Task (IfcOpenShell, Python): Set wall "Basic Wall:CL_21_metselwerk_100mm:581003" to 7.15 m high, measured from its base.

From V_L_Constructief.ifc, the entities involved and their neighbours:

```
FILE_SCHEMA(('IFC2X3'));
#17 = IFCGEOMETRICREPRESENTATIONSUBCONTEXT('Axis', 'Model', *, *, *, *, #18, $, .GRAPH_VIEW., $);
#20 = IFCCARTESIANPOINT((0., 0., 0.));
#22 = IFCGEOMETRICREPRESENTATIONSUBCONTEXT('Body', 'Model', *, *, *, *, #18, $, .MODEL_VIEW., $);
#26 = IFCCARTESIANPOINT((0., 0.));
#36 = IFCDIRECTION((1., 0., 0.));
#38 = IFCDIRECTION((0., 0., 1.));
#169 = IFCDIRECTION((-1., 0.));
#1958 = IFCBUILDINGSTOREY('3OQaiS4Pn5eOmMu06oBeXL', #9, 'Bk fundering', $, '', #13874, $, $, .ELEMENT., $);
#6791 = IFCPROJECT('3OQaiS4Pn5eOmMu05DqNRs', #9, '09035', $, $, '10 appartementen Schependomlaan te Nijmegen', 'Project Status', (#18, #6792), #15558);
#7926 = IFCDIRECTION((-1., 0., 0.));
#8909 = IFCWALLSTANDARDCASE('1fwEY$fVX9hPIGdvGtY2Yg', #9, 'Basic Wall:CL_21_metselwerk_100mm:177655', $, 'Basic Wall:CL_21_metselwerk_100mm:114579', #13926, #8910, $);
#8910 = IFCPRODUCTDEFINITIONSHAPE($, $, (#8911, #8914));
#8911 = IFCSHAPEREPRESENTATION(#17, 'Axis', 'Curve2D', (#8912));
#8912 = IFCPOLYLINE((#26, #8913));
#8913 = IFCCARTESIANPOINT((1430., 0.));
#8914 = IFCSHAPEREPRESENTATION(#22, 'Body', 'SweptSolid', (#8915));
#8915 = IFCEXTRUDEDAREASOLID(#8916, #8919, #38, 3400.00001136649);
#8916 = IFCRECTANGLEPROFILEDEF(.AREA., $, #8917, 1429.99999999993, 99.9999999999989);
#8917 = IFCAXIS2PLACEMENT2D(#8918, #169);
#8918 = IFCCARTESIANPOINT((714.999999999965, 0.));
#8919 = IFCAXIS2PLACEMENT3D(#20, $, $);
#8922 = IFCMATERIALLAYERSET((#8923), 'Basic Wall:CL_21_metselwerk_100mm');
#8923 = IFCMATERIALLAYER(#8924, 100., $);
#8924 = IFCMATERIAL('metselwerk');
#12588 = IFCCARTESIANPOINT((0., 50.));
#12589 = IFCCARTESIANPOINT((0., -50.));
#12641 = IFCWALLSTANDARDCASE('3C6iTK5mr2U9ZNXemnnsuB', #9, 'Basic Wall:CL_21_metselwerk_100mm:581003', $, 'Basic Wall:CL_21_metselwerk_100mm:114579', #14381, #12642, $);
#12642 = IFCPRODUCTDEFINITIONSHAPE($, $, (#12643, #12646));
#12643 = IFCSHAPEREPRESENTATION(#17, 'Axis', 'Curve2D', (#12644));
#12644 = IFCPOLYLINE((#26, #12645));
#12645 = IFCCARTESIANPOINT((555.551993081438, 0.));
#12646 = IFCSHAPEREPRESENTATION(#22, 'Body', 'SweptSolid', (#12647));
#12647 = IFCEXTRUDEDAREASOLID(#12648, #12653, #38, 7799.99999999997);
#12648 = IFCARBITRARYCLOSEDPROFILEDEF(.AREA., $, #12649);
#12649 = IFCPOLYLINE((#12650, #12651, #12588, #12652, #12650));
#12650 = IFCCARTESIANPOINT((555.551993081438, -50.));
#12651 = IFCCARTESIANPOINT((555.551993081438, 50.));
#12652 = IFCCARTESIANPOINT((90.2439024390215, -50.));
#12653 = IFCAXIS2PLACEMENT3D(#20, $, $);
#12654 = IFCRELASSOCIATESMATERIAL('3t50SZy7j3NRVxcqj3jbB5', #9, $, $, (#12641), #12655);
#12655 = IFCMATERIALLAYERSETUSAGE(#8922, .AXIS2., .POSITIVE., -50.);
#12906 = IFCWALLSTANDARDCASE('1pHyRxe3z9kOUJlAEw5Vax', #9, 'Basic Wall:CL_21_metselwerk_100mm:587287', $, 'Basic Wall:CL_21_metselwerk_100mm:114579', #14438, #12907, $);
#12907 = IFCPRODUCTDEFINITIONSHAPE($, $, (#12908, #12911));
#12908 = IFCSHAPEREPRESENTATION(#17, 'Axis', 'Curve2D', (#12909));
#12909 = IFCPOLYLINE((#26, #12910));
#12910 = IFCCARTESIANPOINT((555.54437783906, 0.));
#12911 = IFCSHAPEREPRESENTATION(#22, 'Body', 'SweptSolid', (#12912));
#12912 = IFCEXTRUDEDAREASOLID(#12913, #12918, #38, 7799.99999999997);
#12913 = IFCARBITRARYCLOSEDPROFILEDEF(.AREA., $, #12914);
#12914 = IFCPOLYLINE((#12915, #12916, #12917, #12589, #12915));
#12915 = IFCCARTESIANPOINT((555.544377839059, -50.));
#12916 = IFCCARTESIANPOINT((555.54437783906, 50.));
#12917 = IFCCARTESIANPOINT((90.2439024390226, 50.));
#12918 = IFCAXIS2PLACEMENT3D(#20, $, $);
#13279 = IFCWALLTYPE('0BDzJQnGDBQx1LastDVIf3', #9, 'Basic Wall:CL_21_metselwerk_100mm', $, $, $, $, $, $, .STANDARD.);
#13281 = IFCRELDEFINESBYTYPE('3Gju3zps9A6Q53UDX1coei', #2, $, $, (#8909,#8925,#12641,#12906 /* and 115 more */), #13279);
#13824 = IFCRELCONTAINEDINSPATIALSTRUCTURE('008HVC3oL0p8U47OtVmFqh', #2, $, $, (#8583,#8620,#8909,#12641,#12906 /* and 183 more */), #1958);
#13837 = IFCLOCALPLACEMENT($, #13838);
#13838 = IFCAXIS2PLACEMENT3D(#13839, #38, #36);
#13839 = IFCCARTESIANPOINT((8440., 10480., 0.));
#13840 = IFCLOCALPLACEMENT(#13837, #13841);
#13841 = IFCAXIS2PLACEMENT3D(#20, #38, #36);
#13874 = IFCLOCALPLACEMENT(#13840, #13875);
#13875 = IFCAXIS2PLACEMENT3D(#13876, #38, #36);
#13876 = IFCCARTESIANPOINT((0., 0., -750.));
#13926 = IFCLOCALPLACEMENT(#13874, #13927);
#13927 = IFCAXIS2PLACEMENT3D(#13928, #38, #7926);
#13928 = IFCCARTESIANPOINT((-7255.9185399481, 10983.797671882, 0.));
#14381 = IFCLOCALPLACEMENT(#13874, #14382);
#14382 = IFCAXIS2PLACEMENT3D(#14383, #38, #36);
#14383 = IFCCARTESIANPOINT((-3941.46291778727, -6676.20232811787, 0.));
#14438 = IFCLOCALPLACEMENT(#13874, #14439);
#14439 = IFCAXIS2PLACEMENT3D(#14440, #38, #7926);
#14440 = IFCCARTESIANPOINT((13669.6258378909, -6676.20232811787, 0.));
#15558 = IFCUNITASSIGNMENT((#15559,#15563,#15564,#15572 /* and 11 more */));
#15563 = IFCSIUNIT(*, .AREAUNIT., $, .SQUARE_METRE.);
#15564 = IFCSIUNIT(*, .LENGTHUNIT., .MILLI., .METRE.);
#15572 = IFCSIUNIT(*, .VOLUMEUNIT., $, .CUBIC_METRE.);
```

```python
import ifcopenshell
import ifcopenshell.geom
import ifcopenshell.util.representation
import ifcopenshell.util.shape
import ifcopenshell.util.unit

model = ifcopenshell.open("V_L_Constructief.ifc")
unit_scale = ifcopenshell.util.unit.calculate_unit_scale(model)
settings = ifcopenshell.geom.settings()


def volume(element):
    """Net volume in cubic metres, openings subtracted."""
    shape = ifcopenshell.geom.create_shape(settings, element)
    return ifcopenshell.util.shape.get_volume(shape.geometry)


wall = model.by_guid("3C6iTK5mr2U9ZNXemnnsuB")
before = volume(wall)

body = ifcopenshell.util.representation.get_representation(wall, "Model", "Body")
solid = body.Items[0]
old_height = solid.Depth
solid.Depth = 7.15 / unit_scale
after = volume(wall)

print(f"height {old_height:g} -> {solid.Depth:g}, volume {before:.3f} -> {after:.3f} m3")

model.write("V_L_Constructief_v2.ifc")
```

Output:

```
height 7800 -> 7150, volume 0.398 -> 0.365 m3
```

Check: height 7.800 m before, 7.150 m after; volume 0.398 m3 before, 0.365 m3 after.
